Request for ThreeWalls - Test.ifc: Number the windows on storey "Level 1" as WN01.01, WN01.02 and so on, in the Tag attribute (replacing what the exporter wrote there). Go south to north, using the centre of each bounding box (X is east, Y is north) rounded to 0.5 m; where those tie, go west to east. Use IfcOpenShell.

First a look at what the model holds.

```python
import ifcopenshell
import ifcopenshell.util.element
import ifcopenshell.util.placement

model = ifcopenshell.open("ThreeWalls - Test.ifc")
print(model.schema)
storey = next(s for s in model.by_type("IfcBuildingStorey") if s.Name == "Level 1")
windows = [e for e in ifcopenshell.util.element.get_decomposition(storey) if e.is_a("IfcWindow")]
for e in sorted(windows, key=lambda e: e.id()):
    origin = ifcopenshell.util.placement.get_local_placement(e.ObjectPlacement)[:3, 3]
    print(e.id(), e.Tag, e.Name, origin.round(2) + 0.0, sep=" | ")
```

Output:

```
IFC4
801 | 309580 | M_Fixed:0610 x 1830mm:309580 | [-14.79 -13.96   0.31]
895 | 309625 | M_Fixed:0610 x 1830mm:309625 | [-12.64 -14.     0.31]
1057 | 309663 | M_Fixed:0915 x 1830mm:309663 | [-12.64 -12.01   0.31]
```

```python
import ifcopenshell
import ifcopenshell.geom
import ifcopenshell.util.element
import ifcopenshell.util.shape

model = ifcopenshell.open("ThreeWalls - Test.ifc")
settings = ifcopenshell.geom.settings()
settings.set("use-world-coords", True)


def centre(element):
    shape = ifcopenshell.geom.create_shape(settings, element)
    return ifcopenshell.util.shape.get_bbox_centroid(shape.geometry)


storey = next(s for s in model.by_type("IfcBuildingStorey") if s.Name == "Level 1")
windows = [e for e in ifcopenshell.util.element.get_decomposition(storey) if e.is_a("IfcWindow")]

# Insertion points can sit at a corner or the storey origin, so sort by the geometry (in metres).
centres = {e: centre(e) for e in windows}
windows.sort(key=lambda e: (round(centres[e][1] / 0.5), centres[e][0]))

for i, e in enumerate(windows, start=1):
    number = f"WN01.{i:02d}"
    e.Tag = number
    print(e.id(), number)

model.write("ThreeWalls - Test_rev.ifc")
```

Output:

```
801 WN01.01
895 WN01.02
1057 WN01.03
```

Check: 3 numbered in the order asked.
